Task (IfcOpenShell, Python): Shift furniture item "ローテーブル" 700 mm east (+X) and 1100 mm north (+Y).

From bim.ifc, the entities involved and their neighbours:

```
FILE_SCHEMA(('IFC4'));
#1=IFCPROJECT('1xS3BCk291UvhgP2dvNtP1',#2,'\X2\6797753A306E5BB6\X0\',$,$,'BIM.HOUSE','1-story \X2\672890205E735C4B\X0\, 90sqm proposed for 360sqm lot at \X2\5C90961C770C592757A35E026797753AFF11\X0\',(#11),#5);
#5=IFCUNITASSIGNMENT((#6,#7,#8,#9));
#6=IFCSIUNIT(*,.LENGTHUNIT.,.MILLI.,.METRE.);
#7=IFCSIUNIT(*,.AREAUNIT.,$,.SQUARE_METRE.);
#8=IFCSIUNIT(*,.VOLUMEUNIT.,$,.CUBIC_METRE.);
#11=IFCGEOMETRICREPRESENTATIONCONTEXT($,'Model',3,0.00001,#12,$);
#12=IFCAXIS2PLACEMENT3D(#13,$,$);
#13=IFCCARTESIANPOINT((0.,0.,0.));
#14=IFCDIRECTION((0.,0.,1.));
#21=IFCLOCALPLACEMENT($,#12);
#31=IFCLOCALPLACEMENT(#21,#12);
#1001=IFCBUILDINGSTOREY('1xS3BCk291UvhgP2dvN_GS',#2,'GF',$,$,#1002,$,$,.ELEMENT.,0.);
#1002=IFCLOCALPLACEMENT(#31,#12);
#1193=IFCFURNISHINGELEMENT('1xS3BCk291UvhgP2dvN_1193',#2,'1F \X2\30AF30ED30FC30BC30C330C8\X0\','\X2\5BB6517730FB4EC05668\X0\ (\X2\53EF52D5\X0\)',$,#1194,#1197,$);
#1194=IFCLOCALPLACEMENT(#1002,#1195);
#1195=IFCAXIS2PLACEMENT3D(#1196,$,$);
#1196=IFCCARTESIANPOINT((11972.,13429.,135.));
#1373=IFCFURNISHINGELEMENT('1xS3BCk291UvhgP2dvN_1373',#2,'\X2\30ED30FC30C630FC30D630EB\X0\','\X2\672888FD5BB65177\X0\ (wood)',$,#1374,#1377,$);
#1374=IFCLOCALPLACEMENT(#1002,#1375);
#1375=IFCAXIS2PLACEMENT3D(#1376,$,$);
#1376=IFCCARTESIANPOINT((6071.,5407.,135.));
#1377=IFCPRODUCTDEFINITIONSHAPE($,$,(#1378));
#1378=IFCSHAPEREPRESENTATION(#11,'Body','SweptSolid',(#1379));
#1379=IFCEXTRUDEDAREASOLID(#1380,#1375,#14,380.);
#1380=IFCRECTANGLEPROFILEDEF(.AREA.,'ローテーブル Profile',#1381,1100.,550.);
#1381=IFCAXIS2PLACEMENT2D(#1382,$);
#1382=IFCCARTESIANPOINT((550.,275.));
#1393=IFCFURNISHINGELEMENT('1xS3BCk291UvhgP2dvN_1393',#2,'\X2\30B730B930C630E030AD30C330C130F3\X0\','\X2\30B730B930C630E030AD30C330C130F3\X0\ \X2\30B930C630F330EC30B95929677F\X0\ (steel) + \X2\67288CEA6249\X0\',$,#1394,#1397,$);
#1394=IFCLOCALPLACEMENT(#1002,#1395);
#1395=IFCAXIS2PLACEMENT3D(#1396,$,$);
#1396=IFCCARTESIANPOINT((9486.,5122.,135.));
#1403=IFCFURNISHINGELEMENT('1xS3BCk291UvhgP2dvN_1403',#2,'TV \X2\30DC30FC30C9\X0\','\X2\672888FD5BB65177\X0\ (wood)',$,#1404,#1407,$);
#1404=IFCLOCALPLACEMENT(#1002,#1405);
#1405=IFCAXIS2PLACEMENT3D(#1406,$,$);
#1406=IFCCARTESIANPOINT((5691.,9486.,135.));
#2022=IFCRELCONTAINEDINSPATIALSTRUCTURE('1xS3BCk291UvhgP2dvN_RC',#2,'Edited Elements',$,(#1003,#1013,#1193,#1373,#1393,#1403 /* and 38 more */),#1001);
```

```python
import ifcopenshell
import ifcopenshell.api.geometry
import ifcopenshell.util.placement
import ifcopenshell.util.unit

model = ifcopenshell.open("bim.ifc")
unit_scale = ifcopenshell.util.unit.calculate_unit_scale(model)

item = model.by_id(1373)
matrix = ifcopenshell.util.placement.get_local_placement(item.ObjectPlacement)
matrix[0, 3] += 0.7 / unit_scale
matrix[1, 3] += 1.1 / unit_scale
ifcopenshell.api.geometry.edit_object_placement(model, product=item, matrix=matrix, is_si=False)

print(ifcopenshell.util.placement.get_local_placement(item.ObjectPlacement).round(3) + 0.0)

model.write("bim_edited.ifc")
```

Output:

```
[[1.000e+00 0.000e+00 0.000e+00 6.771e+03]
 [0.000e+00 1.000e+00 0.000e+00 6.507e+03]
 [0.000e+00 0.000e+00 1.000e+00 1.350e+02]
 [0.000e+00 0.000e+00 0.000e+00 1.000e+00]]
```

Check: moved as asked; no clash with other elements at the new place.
